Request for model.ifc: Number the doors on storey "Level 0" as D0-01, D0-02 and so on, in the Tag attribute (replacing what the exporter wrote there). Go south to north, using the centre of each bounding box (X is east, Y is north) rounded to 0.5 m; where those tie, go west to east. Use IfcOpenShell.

First a look at what the model holds.

```python
import ifcopenshell
import ifcopenshell.util.element
import ifcopenshell.util.placement

model = ifcopenshell.open("model.ifc")
print(model.schema)
storey = next(s for s in model.by_type("IfcBuildingStorey") if s.Name == "Level 0")
doors = [e for e in ifcopenshell.util.element.get_decomposition(storey) if e.is_a("IfcDoor")]
for e in sorted(doors, key=lambda e: e.id()):
    origin = ifcopenshell.util.placement.get_local_placement(e.ObjectPlacement)[:3, 3]
    print(e.id(), e.Tag, e.Name, origin.round(2) + 0.0, sep=" | ")
```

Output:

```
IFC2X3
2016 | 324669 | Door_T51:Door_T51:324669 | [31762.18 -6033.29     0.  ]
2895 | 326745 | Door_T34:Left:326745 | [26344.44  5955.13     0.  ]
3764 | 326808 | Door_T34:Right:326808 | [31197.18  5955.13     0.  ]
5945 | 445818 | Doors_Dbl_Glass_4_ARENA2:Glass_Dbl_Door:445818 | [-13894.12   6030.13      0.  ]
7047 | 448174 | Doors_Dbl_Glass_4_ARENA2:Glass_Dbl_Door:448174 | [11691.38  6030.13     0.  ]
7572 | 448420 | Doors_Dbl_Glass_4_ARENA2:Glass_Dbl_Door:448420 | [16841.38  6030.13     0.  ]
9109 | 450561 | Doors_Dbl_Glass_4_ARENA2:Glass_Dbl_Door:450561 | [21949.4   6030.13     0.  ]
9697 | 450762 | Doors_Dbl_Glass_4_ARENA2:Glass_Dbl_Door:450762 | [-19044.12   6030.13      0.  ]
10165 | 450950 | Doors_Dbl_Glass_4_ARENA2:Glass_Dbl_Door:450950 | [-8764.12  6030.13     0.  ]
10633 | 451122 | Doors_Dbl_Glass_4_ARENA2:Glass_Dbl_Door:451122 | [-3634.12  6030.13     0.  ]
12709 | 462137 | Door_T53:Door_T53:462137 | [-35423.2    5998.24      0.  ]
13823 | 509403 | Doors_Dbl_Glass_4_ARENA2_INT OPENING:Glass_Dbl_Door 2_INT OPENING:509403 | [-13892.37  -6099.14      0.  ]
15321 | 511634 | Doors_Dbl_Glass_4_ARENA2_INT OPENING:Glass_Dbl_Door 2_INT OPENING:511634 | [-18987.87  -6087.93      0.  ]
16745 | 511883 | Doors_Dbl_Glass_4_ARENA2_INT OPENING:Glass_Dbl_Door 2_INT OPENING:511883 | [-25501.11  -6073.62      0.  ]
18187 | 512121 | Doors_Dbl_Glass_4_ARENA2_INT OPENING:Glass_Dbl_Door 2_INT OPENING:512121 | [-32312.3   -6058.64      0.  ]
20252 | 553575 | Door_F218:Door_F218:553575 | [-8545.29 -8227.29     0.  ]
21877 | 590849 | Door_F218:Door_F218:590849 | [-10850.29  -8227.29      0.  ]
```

```python
import ifcopenshell
import ifcopenshell.geom
import ifcopenshell.util.element
import ifcopenshell.util.shape

model = ifcopenshell.open("model.ifc")
settings = ifcopenshell.geom.settings()
settings.set("use-world-coords", True)


def centre(element):
    shape = ifcopenshell.geom.create_shape(settings, element)
    return ifcopenshell.util.shape.get_bbox_centroid(shape.geometry)


storey = next(s for s in model.by_type("IfcBuildingStorey") if s.Name == "Level 0")
doors = [e for e in ifcopenshell.util.element.get_decomposition(storey) if e.is_a("IfcDoor")]

# Insertion points can sit at a corner or the storey origin, so sort by the geometry (in metres).
centres = {e: centre(e) for e in doors}
doors.sort(key=lambda e: (round(centres[e][1] / 0.5), centres[e][0]))

for i, e in enumerate(doors, start=1):
    number = f"D0-{i:02d}"
    e.Tag = number
    print(e.id(), number)

model.write("model_v2.ifc")
```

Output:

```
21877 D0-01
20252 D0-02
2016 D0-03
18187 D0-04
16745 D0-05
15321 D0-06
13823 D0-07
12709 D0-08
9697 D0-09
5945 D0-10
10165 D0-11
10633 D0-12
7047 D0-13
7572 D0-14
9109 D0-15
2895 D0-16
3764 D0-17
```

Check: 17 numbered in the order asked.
